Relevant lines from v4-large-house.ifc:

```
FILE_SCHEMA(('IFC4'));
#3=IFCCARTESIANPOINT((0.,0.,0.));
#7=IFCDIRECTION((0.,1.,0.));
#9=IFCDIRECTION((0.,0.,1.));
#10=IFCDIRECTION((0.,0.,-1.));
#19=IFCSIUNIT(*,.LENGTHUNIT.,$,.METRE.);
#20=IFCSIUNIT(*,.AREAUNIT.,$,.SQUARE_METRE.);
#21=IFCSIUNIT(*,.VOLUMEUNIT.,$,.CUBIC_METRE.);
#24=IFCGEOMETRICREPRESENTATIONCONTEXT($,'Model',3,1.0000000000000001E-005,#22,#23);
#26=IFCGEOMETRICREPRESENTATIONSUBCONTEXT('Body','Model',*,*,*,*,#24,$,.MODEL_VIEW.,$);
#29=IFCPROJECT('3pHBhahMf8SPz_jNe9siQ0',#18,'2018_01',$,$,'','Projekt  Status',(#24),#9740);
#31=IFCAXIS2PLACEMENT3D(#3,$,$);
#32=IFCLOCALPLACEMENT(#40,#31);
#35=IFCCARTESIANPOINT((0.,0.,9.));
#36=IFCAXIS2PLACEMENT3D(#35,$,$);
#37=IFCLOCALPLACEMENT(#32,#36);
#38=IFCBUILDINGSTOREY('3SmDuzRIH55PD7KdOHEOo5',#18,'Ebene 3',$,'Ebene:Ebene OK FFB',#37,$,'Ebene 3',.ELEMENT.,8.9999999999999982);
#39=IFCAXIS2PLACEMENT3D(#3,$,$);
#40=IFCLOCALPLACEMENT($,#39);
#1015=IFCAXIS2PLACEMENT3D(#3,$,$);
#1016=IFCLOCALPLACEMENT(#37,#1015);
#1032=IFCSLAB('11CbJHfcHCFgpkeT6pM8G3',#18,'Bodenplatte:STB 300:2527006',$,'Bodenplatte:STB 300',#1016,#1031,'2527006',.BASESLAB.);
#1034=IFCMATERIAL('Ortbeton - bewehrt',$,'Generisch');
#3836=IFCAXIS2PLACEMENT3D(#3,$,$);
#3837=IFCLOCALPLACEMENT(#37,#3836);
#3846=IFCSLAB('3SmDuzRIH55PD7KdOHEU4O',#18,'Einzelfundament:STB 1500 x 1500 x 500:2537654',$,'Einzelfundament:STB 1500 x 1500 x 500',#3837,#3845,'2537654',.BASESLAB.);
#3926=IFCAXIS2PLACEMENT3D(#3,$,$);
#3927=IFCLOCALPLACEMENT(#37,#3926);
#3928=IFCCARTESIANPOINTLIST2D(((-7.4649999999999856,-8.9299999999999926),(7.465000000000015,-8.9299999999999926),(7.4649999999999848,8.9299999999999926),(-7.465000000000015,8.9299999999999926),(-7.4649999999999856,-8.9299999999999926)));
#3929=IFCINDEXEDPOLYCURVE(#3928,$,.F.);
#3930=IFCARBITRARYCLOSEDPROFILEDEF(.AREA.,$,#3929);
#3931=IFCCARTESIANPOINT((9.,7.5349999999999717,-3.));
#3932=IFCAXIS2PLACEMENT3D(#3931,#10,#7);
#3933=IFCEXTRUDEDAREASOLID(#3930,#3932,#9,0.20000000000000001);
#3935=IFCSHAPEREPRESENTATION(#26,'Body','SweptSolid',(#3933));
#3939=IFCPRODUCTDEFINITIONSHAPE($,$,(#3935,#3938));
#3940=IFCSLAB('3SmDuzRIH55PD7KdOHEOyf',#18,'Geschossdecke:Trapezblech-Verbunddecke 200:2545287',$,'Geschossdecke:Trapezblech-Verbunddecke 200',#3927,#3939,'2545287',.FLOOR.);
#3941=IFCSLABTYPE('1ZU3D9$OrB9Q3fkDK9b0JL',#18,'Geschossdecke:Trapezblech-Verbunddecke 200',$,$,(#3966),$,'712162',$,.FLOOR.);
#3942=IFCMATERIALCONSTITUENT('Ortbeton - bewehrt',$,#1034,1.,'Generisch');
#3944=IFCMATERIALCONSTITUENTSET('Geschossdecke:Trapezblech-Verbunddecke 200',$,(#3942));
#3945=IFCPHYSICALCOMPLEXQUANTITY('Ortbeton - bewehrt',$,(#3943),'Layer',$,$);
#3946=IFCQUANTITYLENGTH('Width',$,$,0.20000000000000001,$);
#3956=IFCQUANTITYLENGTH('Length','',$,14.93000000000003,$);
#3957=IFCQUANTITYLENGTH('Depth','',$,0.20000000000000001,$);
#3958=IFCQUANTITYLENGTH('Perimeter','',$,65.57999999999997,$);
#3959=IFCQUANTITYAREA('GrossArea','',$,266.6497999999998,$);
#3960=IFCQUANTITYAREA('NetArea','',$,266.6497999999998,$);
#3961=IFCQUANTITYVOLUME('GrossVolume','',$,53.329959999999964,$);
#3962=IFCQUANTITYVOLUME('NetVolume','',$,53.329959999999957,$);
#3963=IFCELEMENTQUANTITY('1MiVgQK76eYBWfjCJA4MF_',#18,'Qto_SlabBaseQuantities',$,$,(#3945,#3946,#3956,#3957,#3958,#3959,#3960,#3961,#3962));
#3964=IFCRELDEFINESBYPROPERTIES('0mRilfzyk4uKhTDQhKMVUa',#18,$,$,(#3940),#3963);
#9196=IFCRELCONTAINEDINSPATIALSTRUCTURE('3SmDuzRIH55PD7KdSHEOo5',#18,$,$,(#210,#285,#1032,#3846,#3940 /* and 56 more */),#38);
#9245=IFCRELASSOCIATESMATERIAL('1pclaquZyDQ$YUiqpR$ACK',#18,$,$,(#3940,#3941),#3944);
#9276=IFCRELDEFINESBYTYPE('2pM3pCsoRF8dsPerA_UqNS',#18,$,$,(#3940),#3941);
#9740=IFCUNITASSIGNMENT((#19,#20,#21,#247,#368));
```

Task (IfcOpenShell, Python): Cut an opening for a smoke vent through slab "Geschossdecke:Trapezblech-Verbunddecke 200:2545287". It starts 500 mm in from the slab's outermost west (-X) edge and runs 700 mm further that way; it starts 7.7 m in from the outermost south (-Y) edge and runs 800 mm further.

```python
import numpy as np
import ifcopenshell
import ifcopenshell.api.feature
import ifcopenshell.api.geometry
import ifcopenshell.api.pset
import ifcopenshell.api.root
import ifcopenshell.geom
import ifcopenshell.util.element
import ifcopenshell.util.placement
import ifcopenshell.util.representation
import ifcopenshell.util.shape
import ifcopenshell.util.unit

model = ifcopenshell.open("v4-large-house.ifc")
unit_scale = ifcopenshell.util.unit.calculate_unit_scale(model)
area_scale = ifcopenshell.util.unit.calculate_unit_scale(model, "AREAUNIT")
volume_scale = ifcopenshell.util.unit.calculate_unit_scale(model, "VOLUMEUNIT")
settings = ifcopenshell.geom.settings()


def volume(element):
    """Net volume in cubic metres, openings subtracted."""
    shape = ifcopenshell.geom.create_shape(settings, element)
    return ifcopenshell.util.shape.get_volume(shape.geometry)


slab = model.by_guid("3SmDuzRIH55PD7KdOHEOyf")
before = volume(slab)

# Extent in the slab's own axes, in metres. The edges named are its -X and -Y sides.
slab_shape = ifcopenshell.geom.create_shape(settings, slab)
vertices = ifcopenshell.util.shape.get_vertices(slab_shape.geometry)
x_min, y_min, bottom = vertices.min(axis=0)
top = vertices[:, 2].max()

opening = ifcopenshell.api.root.create_entity(model, ifc_class="IfcOpeningElement", name="Smoke vent opening", predefined_type="OPENING")
context = ifcopenshell.util.representation.get_context(model, "Model", "Body", "MODEL_VIEW")
width, depth = 0.7, 0.8
outline = [(0.0, 0.0), (width, 0.0), (width, depth), (0.0, depth), (0.0, 0.0)]
# Overshoot both faces by 50 mm so the cut is clean.
shape = ifcopenshell.api.geometry.add_slab_representation(
    model, context=context, depth=top - bottom + 0.1, polyline=outline
)
ifcopenshell.api.geometry.assign_representation(model, product=opening, representation=shape)

matrix = ifcopenshell.util.placement.get_local_placement(slab.ObjectPlacement)
matrix[:, 3] = matrix @ np.append(np.array([x_min + 0.5, y_min + 7.7, bottom - 0.05]) / unit_scale, 1.0)
ifcopenshell.api.geometry.edit_object_placement(model, product=opening, matrix=matrix, is_si=False)
ifcopenshell.api.feature.add_feature(model, feature=opening, element=slab)

after = volume(slab)

# Update the slab's stored quantities.
qto = model.by_id(ifcopenshell.util.element.get_pset(slab, "Qto_SlabBaseQuantities", should_inherit=False)["id"])
ifcopenshell.api.pset.edit_qto(model, qto=qto, properties={
    "NetArea": after / (top - bottom) / area_scale,
    "NetVolume": after / volume_scale,
})

print(f"slab volume {before:.3f} -> {after:.3f} m3")

model.write("v4-large-house_rev.ifc")
```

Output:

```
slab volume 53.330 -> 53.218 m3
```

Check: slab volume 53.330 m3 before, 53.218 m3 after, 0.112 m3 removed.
